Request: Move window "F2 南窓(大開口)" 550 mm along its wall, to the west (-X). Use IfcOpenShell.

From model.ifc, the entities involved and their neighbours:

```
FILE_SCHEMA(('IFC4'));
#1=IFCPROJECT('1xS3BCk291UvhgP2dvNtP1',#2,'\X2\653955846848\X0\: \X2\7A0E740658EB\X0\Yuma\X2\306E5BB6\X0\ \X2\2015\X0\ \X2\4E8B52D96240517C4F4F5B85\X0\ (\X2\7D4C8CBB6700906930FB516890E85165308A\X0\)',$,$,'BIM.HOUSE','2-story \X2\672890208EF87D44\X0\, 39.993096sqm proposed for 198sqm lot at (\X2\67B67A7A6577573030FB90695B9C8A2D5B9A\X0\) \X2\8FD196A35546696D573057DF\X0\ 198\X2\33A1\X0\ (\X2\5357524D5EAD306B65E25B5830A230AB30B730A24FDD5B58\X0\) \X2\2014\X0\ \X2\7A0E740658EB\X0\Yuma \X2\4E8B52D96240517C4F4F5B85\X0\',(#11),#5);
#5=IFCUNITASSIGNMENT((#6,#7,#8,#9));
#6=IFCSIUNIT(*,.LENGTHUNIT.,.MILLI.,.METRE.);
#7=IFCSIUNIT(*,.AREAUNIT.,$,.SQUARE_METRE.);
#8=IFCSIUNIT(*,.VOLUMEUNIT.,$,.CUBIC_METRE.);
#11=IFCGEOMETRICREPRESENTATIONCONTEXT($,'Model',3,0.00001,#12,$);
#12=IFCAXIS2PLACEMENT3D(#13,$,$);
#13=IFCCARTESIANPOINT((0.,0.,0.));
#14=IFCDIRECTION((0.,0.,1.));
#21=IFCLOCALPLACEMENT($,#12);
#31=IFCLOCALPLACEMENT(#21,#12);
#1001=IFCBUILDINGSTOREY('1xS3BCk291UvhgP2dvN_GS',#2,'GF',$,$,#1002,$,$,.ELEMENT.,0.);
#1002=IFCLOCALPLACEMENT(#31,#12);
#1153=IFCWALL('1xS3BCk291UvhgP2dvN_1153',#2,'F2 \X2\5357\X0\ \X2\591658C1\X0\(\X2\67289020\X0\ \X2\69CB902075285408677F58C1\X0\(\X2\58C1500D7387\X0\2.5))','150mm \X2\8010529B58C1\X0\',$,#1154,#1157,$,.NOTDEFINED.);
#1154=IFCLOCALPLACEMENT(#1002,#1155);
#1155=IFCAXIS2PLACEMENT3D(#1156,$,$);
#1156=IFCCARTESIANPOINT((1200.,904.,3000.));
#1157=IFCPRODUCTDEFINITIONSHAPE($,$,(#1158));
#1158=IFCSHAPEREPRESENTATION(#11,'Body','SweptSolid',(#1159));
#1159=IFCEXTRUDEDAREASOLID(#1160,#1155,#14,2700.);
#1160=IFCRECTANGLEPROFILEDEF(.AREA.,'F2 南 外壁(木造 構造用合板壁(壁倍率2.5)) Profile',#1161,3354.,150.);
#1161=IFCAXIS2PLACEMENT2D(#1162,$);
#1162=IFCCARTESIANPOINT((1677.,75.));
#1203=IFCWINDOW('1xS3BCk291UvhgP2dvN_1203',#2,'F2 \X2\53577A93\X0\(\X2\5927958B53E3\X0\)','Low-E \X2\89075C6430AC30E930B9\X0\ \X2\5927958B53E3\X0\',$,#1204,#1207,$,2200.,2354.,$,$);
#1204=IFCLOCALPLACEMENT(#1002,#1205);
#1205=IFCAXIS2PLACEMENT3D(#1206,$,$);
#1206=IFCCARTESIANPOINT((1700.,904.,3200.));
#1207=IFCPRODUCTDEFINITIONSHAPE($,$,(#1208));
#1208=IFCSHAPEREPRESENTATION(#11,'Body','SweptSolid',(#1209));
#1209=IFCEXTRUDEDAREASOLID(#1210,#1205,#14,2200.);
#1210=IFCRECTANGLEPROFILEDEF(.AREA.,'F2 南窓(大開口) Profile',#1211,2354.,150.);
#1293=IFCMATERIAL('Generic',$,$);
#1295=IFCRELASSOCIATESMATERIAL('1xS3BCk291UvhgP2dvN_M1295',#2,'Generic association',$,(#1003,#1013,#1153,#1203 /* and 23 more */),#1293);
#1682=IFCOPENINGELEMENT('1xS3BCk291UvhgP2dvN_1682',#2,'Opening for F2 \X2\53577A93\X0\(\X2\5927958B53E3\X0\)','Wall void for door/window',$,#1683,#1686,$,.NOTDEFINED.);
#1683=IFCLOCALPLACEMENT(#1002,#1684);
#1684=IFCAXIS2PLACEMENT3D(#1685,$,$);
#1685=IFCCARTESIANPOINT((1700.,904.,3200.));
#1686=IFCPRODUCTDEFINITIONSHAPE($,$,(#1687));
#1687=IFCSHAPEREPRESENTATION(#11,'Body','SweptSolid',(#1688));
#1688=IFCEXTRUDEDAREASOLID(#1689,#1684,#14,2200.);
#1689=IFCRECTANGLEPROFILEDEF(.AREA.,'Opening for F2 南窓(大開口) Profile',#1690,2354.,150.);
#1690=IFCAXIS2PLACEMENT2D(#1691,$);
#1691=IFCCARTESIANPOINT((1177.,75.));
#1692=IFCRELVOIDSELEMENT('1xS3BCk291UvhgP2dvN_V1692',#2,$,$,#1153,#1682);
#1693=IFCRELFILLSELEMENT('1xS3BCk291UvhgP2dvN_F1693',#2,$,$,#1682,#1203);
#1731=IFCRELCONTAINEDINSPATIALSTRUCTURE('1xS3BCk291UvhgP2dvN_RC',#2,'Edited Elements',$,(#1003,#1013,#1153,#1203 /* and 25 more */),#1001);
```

```python
import ifcopenshell
import ifcopenshell.api.geometry
import ifcopenshell.util.placement

model = ifcopenshell.open("model.ifc")

window = model.by_id(1203)
opening = window.FillsVoids[0].RelatingOpeningElement
wall = opening.VoidsElements[0].RelatingBuildingElement

wall_matrix = ifcopenshell.util.placement.get_local_placement(wall.ObjectPlacement)
shift = wall_matrix[:3, 0] * -550.0
before = ifcopenshell.util.placement.get_local_placement(window.ObjectPlacement)[:3, 3].copy()

# The window is not placed relative to its opening, so move both.
for product in (opening, window):
    matrix = ifcopenshell.util.placement.get_local_placement(product.ObjectPlacement)
    matrix[:3, 3] += shift
    ifcopenshell.api.geometry.edit_object_placement(model, product=product, matrix=matrix, is_si=False)

after = ifcopenshell.util.placement.get_local_placement(window.ObjectPlacement)[:3, 3]
print("window moved by", (after - before).round(3) + 0.0)

model.write("model_edited.ifc")
```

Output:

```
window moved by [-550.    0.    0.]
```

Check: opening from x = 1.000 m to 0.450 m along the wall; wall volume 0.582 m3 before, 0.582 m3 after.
